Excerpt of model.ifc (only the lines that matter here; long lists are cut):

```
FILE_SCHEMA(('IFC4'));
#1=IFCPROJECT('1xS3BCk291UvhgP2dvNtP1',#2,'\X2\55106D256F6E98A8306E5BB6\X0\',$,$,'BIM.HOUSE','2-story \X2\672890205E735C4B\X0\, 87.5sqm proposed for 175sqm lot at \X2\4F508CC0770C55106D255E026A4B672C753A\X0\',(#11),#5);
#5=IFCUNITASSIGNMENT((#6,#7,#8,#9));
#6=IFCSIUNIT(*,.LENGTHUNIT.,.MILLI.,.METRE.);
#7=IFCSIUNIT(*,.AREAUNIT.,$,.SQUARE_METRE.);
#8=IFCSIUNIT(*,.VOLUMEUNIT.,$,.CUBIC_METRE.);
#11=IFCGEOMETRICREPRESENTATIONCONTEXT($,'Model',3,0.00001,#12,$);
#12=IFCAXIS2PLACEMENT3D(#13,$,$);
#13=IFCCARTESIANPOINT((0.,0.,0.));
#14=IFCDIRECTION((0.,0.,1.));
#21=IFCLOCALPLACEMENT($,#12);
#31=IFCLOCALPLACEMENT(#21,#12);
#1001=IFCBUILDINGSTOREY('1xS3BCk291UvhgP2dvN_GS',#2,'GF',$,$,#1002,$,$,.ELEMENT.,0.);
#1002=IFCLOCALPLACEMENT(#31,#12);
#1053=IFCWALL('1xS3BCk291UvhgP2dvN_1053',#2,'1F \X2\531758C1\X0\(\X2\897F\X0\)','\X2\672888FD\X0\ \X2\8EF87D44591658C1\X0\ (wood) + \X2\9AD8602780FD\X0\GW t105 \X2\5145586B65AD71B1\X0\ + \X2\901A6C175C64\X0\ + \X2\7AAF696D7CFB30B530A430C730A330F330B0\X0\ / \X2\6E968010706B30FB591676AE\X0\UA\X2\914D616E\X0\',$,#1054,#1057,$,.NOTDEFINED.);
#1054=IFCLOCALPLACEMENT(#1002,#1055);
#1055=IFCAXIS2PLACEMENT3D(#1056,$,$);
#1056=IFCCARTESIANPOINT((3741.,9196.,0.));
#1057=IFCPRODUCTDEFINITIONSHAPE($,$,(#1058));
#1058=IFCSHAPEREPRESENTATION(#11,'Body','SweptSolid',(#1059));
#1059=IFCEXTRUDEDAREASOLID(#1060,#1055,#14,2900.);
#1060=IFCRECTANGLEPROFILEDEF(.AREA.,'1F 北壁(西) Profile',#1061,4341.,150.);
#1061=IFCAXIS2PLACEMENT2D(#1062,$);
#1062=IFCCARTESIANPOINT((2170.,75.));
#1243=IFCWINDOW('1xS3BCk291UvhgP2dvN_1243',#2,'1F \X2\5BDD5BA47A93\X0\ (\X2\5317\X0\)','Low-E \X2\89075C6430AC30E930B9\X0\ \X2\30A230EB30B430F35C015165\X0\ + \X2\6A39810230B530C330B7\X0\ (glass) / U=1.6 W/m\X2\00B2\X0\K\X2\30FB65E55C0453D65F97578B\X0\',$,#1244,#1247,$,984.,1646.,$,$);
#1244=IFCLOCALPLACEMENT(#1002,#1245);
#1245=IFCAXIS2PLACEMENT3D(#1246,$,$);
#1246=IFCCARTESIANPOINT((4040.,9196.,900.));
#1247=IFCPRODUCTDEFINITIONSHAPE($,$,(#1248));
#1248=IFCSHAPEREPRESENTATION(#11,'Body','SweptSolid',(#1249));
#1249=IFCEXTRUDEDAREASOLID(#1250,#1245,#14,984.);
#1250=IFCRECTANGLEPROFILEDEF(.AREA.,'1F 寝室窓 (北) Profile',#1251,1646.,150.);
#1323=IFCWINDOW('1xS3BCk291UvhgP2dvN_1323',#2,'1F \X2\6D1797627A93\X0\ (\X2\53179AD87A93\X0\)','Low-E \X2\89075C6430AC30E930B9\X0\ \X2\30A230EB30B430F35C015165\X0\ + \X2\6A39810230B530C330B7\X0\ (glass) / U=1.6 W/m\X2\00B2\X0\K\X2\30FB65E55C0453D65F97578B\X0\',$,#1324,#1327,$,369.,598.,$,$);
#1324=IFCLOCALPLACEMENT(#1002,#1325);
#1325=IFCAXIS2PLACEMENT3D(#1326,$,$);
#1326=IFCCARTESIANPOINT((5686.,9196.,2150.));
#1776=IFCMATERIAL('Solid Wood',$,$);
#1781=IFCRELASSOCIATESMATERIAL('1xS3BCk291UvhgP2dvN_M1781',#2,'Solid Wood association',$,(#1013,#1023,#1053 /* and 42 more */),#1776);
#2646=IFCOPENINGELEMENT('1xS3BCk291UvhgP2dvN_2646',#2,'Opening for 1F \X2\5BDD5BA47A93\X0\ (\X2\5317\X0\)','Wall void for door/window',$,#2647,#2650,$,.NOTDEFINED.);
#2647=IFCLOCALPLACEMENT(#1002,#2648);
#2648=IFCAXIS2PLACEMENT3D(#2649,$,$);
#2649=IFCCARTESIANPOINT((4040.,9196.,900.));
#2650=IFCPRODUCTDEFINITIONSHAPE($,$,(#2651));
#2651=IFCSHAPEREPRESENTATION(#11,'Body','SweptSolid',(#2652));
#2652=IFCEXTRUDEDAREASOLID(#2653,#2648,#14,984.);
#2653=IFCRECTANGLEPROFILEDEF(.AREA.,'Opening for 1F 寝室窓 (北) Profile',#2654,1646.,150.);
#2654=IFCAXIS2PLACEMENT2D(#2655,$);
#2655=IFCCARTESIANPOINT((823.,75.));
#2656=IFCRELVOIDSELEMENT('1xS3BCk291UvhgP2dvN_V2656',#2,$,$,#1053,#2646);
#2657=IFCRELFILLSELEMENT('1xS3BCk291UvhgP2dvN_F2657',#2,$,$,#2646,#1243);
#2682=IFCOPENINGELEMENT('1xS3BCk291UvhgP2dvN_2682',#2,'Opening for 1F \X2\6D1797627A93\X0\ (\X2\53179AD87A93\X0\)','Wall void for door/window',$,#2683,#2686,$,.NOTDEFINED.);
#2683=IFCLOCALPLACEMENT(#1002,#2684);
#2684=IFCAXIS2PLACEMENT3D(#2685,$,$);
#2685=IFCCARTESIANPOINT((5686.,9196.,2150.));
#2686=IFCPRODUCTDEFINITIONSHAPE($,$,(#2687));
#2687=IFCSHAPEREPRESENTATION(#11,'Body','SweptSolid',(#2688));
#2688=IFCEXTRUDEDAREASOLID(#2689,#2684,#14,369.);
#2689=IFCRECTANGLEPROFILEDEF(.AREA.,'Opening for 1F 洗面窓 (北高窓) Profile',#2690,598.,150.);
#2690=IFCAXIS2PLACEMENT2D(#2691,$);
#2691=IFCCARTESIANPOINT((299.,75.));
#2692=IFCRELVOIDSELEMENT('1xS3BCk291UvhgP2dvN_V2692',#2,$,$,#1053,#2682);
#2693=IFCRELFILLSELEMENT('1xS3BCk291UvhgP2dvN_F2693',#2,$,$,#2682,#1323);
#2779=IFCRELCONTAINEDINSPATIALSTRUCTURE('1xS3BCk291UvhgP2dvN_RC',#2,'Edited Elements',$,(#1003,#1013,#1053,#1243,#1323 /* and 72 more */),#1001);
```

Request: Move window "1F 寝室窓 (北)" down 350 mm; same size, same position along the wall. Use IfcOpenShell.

```python
import numpy as np
import ifcopenshell
import ifcopenshell.api.geometry
import ifcopenshell.util.placement
import ifcopenshell.util.unit

model = ifcopenshell.open("model.ifc")
unit_scale = ifcopenshell.util.unit.calculate_unit_scale(model)

window = model.by_guid("1xS3BCk291UvhgP2dvN_1243")
opening = window.FillsVoids[0].RelatingOpeningElement
dz = -0.35 / unit_scale

shift = np.array([0.0, 0.0, dz])
# The window is not placed relative to its opening, so move both.
for product in (opening, window):
    matrix = ifcopenshell.util.placement.get_local_placement(product.ObjectPlacement)
    matrix[:3, 3] += shift
    ifcopenshell.api.geometry.edit_object_placement(model, product=product, matrix=matrix, is_si=False)

print(f"moved by {dz * unit_scale:+.3f} m")

model.write("model_v2.ifc")
```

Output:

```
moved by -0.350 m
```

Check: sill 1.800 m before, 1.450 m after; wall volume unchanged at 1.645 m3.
